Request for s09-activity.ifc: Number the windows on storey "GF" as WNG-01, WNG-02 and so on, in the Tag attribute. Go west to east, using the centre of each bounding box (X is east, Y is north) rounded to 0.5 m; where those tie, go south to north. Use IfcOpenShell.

First a look at what the model holds.

```python
import ifcopenshell
import ifcopenshell.util.element
import ifcopenshell.util.placement

model = ifcopenshell.open("s09-activity.ifc")
print(model.schema)
storey = next(s for s in model.by_type("IfcBuildingStorey") if s.Name == "GF")
windows = [e for e in ifcopenshell.util.element.get_decomposition(storey) if e.is_a("IfcWindow")]
for e in sorted(windows, key=lambda e: e.id()):
    origin = ifcopenshell.util.placement.get_local_placement(e.ObjectPlacement)[:3, 3]
    print(e.id(), e.Tag, e.Name, origin.round(2) + 0.0, sep=" | ")
```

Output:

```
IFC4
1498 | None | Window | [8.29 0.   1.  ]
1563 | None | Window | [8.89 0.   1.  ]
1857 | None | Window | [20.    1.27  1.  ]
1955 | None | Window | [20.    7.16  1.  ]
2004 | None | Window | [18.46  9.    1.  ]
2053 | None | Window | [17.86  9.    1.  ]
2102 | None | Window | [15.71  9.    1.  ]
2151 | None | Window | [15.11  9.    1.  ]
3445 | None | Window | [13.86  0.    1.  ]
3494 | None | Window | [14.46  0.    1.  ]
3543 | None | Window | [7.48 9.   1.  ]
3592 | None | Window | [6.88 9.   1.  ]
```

```python
import ifcopenshell
import ifcopenshell.geom
import ifcopenshell.util.element
import ifcopenshell.util.shape

model = ifcopenshell.open("s09-activity.ifc")
settings = ifcopenshell.geom.settings()
settings.set("use-world-coords", True)


def centre(element):
    shape = ifcopenshell.geom.create_shape(settings, element)
    return ifcopenshell.util.shape.get_bbox_centroid(shape.geometry)


storey = next(s for s in model.by_type("IfcBuildingStorey") if s.Name == "GF")
windows = [e for e in ifcopenshell.util.element.get_decomposition(storey) if e.is_a("IfcWindow")]

# Insertion points can sit at a corner or the storey origin, so sort by the geometry (in metres).
centres = {e: centre(e) for e in windows}
windows.sort(key=lambda e: (round(centres[e][0] / 0.5), centres[e][1]))

for i, e in enumerate(windows, start=1):
    number = f"WNG-{i:02d}"
    e.Tag = number
    print(e.id(), number)

model.write("s09-activity_rev.ifc")
```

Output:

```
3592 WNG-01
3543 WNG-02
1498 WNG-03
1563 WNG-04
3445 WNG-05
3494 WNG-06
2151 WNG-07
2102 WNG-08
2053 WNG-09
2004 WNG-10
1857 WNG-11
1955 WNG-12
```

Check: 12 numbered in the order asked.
